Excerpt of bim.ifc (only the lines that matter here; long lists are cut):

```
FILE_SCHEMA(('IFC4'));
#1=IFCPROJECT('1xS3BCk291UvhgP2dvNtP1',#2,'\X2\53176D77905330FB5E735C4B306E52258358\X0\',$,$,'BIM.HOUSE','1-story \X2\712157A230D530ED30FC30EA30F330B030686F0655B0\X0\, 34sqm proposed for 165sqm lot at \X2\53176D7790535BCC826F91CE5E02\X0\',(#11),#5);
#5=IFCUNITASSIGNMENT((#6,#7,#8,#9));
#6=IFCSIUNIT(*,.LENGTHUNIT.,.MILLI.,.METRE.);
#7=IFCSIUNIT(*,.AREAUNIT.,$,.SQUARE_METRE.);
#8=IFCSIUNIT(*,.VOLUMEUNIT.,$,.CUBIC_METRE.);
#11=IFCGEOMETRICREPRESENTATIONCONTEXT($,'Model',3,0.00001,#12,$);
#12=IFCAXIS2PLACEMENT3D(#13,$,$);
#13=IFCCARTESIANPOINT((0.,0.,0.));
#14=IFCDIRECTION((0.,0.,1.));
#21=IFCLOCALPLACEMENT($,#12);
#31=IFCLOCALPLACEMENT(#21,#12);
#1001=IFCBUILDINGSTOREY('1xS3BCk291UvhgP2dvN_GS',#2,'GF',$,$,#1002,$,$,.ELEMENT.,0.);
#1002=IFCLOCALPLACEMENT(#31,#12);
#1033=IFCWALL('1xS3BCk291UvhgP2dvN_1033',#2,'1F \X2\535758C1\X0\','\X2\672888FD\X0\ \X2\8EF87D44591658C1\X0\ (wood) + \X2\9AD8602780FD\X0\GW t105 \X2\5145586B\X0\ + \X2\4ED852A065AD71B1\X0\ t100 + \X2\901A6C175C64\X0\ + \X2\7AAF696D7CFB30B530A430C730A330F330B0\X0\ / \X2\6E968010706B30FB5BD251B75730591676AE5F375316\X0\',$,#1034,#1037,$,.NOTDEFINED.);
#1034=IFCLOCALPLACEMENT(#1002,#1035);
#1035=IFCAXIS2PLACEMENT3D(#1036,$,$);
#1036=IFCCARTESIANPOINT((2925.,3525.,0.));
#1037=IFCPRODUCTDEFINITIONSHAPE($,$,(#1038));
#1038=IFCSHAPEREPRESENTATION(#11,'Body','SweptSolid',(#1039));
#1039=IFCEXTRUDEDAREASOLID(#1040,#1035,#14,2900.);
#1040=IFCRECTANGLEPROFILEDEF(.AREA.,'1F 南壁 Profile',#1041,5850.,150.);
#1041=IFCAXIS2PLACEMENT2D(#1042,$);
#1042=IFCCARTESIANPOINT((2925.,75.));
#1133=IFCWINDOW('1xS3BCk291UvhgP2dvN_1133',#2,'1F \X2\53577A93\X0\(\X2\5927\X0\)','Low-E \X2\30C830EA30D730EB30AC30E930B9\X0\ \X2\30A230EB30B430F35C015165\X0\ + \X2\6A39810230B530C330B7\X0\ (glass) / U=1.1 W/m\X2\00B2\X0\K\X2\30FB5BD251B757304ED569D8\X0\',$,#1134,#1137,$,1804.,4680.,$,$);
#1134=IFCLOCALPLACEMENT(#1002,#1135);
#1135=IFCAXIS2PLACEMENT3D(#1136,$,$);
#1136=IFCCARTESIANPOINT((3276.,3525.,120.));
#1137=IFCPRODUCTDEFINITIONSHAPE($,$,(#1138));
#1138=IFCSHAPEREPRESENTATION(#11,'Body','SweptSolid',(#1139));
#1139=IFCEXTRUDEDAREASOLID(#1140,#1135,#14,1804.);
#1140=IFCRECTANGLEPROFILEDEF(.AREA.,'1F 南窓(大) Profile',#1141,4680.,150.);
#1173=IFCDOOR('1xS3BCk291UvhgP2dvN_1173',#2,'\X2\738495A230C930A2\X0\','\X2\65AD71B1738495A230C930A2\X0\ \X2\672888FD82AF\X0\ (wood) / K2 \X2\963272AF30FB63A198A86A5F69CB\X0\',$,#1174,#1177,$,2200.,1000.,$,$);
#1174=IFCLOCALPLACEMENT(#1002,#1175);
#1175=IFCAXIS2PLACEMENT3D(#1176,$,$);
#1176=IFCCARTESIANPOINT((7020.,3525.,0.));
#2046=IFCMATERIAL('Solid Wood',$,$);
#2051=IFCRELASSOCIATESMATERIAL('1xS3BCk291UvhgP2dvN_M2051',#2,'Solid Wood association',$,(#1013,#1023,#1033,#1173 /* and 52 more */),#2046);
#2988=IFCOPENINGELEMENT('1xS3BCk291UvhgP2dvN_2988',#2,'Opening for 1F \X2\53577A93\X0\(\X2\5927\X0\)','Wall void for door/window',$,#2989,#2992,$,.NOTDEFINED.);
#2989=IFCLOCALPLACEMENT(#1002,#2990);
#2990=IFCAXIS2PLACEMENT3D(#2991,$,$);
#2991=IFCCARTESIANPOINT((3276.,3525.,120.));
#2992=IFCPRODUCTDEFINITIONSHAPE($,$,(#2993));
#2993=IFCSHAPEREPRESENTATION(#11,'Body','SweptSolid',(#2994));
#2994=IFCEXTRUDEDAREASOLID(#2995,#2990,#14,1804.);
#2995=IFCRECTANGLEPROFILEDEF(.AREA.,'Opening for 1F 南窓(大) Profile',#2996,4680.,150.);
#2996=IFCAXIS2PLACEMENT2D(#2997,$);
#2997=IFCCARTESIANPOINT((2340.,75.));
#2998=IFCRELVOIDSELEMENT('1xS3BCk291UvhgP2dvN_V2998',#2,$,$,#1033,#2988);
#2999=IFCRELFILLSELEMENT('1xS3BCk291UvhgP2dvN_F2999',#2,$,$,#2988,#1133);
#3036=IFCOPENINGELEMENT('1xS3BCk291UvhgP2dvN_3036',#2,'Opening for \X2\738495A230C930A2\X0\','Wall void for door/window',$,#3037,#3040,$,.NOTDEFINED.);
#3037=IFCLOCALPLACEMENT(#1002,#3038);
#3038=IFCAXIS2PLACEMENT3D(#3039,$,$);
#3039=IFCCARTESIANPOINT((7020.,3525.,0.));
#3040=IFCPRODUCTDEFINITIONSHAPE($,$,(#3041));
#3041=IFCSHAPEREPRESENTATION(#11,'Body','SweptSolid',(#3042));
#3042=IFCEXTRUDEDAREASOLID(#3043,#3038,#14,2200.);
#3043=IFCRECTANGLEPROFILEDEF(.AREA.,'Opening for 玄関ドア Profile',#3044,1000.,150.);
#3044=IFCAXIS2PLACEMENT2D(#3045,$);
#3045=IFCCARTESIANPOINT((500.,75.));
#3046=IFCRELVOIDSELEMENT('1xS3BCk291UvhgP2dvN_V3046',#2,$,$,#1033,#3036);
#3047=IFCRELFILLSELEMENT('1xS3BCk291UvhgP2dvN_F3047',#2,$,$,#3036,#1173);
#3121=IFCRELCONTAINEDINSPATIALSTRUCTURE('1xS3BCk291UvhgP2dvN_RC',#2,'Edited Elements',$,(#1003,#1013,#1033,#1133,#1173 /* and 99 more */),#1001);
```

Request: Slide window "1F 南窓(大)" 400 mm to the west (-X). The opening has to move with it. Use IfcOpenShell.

```python
import ifcopenshell
import ifcopenshell.api.geometry
import ifcopenshell.util.placement

model = ifcopenshell.open("bim.ifc")

window = model.by_guid("1xS3BCk291UvhgP2dvN_1133")
opening = window.FillsVoids[0].RelatingOpeningElement
wall = opening.VoidsElements[0].RelatingBuildingElement

wall_matrix = ifcopenshell.util.placement.get_local_placement(wall.ObjectPlacement)
shift = wall_matrix[:3, 0] * -400.0
before = ifcopenshell.util.placement.get_local_placement(window.ObjectPlacement)[:3, 3].copy()

# The window is not placed relative to its opening, so move both.
for product in (opening, window):
    matrix = ifcopenshell.util.placement.get_local_placement(product.ObjectPlacement)
    matrix[:3, 3] += shift
    ifcopenshell.api.geometry.edit_object_placement(model, product=product, matrix=matrix, is_si=False)

after = ifcopenshell.util.placement.get_local_placement(window.ObjectPlacement)[:3, 3]
print("window moved by", (after - before).round(3) + 0.0)

model.write("bim_edited.ifc")
```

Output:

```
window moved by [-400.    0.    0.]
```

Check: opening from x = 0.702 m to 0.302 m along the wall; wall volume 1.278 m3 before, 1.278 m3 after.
